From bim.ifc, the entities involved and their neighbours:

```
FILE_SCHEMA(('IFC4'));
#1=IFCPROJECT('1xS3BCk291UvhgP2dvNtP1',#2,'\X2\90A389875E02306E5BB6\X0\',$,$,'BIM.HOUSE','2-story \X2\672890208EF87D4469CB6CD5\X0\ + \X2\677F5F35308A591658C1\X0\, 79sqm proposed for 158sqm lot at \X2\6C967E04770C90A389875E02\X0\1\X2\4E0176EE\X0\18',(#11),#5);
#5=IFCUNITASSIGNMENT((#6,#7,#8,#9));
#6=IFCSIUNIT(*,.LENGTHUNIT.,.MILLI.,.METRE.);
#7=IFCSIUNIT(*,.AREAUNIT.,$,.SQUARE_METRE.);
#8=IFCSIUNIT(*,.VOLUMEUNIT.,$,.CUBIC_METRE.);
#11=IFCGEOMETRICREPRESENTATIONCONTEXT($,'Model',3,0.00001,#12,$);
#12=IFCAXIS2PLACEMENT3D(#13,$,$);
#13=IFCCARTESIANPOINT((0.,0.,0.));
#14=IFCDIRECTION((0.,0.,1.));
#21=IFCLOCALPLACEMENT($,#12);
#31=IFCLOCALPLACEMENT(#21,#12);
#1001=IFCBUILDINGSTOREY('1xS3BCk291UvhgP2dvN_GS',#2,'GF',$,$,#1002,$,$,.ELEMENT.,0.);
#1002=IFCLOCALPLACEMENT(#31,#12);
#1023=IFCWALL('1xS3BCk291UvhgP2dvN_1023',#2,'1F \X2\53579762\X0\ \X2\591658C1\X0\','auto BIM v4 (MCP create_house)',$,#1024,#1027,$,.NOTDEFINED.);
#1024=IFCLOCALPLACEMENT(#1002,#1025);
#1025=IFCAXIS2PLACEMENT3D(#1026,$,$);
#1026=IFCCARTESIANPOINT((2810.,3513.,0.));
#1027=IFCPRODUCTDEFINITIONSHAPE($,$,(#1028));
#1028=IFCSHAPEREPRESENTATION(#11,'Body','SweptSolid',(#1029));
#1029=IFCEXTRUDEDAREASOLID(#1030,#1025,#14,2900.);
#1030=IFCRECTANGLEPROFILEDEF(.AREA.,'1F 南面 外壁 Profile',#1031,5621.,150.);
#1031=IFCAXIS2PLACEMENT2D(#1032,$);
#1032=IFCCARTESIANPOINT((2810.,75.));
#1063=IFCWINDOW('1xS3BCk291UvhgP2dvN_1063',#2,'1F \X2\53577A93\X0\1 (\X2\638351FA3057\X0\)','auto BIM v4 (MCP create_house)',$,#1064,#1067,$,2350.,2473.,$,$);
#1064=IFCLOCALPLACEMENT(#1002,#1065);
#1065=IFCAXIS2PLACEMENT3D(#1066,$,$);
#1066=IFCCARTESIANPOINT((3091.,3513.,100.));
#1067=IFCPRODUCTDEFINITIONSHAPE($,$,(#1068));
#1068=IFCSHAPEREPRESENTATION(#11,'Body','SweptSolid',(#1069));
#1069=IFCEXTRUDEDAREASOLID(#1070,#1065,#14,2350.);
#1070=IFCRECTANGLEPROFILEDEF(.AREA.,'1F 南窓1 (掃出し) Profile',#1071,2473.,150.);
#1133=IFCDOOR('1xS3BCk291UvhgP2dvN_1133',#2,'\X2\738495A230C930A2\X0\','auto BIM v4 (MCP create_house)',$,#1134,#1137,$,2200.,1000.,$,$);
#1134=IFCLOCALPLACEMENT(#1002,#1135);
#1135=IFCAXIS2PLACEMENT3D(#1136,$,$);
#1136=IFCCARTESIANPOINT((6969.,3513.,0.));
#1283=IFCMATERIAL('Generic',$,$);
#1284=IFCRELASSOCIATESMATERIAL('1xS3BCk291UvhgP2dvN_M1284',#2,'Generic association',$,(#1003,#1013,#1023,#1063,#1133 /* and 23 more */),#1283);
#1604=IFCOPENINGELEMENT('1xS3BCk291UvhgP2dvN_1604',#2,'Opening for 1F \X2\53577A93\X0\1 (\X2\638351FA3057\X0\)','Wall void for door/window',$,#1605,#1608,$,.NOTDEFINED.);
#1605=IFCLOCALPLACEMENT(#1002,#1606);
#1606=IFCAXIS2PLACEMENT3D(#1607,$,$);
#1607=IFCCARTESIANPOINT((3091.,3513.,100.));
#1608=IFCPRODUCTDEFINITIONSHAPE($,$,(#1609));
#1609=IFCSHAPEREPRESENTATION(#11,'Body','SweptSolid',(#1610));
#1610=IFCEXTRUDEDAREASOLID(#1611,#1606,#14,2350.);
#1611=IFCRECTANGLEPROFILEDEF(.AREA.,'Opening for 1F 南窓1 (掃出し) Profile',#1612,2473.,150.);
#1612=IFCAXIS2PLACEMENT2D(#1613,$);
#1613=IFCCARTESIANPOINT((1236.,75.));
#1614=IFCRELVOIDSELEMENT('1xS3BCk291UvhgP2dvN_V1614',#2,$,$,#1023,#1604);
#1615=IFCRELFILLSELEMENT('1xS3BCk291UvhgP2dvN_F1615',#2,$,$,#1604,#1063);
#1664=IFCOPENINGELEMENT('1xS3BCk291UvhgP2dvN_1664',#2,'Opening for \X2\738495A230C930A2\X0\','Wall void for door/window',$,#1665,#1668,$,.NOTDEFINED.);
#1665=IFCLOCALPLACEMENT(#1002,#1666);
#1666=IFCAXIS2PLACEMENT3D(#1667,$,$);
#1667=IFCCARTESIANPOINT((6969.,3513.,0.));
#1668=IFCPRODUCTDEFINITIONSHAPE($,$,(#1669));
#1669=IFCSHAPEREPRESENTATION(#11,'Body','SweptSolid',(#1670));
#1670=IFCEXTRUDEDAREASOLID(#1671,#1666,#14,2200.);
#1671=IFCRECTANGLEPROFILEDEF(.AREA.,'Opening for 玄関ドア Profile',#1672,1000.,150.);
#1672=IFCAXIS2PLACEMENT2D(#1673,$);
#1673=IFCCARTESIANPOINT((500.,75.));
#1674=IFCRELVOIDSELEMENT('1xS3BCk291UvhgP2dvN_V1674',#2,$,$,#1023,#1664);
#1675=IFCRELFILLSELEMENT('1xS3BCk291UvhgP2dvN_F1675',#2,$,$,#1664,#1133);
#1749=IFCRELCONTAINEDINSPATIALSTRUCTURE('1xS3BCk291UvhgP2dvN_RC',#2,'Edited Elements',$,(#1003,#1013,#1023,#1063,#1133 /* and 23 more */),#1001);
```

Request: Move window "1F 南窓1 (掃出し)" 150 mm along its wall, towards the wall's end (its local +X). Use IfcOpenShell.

```python
import ifcopenshell
import ifcopenshell.api.geometry
import ifcopenshell.util.placement
import ifcopenshell.util.unit

model = ifcopenshell.open("bim.ifc")
unit_scale = ifcopenshell.util.unit.calculate_unit_scale(model)

window = model.by_id(1063)
opening = window.FillsVoids[0].RelatingOpeningElement
wall = opening.VoidsElements[0].RelatingBuildingElement

wall_matrix = ifcopenshell.util.placement.get_local_placement(wall.ObjectPlacement)
shift = wall_matrix[:3, 0] * 0.15 / unit_scale
before = ifcopenshell.util.placement.get_local_placement(window.ObjectPlacement)[:3, 3].copy()

# The window is not placed relative to its opening, so move both.
for product in (opening, window):
    matrix = ifcopenshell.util.placement.get_local_placement(product.ObjectPlacement)
    matrix[:3, 3] += shift
    ifcopenshell.api.geometry.edit_object_placement(model, product=product, matrix=matrix, is_si=False)

after = ifcopenshell.util.placement.get_local_placement(window.ObjectPlacement)[:3, 3]
print("window moved by", (after - before).round(3) + 0.0)

model.write("bim_rev.ifc")
```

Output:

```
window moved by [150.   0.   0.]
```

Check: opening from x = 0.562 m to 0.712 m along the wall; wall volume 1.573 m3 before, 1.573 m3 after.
